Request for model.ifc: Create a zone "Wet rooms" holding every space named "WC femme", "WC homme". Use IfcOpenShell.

First a look at what the model holds.

```python
import ifcopenshell

model = ifcopenshell.open("model.ifc")
print(model.schema)
seen = {}
for space in model.by_type("IfcSpace"):
    seen[space.LongName] = seen.get(space.LongName, 0) + 1
for name, count in sorted(seen.items(), key=str):
    print(count, "x", name)
print("zones:", [z.Name for z in model.by_type("IfcZone")][:20])
```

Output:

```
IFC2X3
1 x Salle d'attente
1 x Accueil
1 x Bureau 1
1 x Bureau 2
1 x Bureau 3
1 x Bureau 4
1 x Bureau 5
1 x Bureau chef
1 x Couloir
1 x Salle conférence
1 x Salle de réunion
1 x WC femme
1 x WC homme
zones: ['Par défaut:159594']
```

```python
import ifcopenshell
import ifcopenshell.api.group
import ifcopenshell.api.root

model = ifcopenshell.open("model.ifc")

names = {"WC femme", "WC homme"}
spaces = [s for s in model.by_type("IfcSpace") if s.LongName in names]

zone = ifcopenshell.api.root.create_entity(model, ifc_class="IfcZone", name="Wet rooms")
ifcopenshell.api.group.assign_group(model, products=spaces, group=zone)
print(len(spaces), "spaces in", zone.Name)

model.write("model_v2.ifc")
```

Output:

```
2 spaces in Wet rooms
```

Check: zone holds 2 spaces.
